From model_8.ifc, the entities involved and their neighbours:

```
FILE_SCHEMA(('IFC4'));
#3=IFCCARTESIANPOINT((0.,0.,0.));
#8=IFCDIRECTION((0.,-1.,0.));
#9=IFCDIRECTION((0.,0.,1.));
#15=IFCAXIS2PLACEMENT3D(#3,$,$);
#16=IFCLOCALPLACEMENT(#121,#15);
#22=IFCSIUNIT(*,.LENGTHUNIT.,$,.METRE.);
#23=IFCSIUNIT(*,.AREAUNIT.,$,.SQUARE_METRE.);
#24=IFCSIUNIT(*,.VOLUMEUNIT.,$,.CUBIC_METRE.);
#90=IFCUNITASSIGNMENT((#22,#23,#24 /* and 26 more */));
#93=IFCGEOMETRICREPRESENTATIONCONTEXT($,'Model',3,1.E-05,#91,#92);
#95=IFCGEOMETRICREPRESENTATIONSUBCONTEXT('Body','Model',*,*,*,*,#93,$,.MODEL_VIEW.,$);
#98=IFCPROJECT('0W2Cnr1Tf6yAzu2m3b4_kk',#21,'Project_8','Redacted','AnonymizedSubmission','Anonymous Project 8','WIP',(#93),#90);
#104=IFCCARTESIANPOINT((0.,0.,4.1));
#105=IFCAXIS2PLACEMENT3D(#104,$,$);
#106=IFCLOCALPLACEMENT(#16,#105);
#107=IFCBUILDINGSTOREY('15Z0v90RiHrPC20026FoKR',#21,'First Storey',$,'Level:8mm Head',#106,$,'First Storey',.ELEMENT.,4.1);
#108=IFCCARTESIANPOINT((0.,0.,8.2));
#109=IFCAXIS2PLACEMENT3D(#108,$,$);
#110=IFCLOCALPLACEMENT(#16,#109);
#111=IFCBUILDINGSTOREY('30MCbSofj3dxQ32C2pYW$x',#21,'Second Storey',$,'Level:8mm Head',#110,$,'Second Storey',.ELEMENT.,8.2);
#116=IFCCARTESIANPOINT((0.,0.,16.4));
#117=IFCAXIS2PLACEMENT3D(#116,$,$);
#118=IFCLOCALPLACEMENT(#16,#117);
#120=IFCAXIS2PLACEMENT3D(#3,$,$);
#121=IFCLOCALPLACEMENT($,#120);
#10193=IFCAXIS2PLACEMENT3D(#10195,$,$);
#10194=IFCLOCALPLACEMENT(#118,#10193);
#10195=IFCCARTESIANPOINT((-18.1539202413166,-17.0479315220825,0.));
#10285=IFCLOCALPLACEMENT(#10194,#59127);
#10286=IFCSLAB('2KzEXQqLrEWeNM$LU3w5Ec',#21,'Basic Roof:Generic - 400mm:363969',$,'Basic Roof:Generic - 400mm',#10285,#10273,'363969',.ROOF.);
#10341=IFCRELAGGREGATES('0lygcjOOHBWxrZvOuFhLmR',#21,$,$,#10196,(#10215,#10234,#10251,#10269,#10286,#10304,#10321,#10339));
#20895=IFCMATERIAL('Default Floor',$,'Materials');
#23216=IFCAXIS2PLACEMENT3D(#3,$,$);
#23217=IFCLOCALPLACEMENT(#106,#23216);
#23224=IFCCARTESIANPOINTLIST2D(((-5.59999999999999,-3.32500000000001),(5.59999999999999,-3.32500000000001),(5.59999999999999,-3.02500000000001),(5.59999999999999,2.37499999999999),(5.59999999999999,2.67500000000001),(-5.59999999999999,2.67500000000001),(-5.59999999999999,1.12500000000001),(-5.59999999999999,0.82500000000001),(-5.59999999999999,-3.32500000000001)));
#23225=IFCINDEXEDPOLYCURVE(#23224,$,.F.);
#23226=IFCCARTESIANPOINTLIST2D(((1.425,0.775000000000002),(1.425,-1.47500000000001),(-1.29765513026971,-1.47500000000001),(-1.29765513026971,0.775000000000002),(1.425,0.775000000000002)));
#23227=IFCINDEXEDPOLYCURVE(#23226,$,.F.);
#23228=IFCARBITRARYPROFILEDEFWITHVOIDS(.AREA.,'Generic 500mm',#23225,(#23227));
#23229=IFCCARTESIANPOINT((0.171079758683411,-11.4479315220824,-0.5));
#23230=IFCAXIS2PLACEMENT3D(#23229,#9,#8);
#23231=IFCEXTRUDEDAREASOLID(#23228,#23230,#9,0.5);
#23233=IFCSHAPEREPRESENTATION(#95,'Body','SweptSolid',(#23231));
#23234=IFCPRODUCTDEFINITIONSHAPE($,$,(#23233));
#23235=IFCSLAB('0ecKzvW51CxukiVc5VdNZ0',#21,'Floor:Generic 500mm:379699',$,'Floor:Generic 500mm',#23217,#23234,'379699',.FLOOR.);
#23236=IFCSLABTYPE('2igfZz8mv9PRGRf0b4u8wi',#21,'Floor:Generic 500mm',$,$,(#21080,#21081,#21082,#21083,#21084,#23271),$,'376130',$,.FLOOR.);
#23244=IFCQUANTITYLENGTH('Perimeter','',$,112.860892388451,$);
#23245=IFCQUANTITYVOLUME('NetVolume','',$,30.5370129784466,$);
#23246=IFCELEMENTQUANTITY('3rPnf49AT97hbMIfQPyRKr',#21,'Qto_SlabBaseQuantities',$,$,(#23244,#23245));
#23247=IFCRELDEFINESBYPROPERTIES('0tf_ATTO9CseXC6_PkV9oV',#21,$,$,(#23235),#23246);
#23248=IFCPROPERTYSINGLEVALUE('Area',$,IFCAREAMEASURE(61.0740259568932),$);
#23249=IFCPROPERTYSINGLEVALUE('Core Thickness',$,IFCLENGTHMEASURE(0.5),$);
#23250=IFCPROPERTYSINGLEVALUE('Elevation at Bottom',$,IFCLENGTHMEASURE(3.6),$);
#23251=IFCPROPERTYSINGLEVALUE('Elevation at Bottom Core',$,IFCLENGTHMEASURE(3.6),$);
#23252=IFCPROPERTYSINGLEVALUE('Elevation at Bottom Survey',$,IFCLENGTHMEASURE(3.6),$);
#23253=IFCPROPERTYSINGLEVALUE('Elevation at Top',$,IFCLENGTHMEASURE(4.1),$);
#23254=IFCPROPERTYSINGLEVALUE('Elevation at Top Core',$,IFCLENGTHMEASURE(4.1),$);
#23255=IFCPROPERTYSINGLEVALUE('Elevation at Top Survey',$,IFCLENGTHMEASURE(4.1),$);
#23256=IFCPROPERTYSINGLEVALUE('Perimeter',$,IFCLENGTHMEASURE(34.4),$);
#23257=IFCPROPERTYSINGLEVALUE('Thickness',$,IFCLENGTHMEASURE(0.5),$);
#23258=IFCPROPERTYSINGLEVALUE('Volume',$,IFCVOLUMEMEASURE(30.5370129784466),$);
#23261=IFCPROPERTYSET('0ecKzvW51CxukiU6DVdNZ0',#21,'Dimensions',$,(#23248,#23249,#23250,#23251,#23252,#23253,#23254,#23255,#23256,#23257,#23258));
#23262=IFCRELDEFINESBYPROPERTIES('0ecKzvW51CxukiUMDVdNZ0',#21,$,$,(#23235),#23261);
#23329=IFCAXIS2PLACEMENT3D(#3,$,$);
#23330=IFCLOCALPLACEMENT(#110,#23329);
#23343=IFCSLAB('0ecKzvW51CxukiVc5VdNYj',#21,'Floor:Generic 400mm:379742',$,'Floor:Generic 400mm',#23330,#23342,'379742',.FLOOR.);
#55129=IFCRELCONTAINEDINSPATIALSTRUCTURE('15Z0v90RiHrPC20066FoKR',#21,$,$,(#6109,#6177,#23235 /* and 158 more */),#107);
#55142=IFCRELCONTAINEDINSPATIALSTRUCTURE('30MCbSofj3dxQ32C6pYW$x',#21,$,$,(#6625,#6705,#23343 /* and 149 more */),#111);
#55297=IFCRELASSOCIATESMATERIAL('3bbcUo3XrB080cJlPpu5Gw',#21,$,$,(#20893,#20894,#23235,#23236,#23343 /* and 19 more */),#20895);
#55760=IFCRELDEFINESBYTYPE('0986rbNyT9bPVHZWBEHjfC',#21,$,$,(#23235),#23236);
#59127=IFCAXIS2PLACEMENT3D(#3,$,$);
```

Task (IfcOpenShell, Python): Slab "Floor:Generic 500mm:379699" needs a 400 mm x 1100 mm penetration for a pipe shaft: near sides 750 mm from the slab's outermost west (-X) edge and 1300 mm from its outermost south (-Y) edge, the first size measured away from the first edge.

```python
import numpy as np
import ifcopenshell
import ifcopenshell.api.feature
import ifcopenshell.api.geometry
import ifcopenshell.api.pset
import ifcopenshell.api.root
import ifcopenshell.geom
import ifcopenshell.util.element
import ifcopenshell.util.placement
import ifcopenshell.util.representation
import ifcopenshell.util.shape
import ifcopenshell.util.unit

model = ifcopenshell.open("model_8.ifc")
unit_scale = ifcopenshell.util.unit.calculate_unit_scale(model)
area_scale = ifcopenshell.util.unit.calculate_unit_scale(model, "AREAUNIT")
volume_scale = ifcopenshell.util.unit.calculate_unit_scale(model, "VOLUMEUNIT")
settings = ifcopenshell.geom.settings()


def volume(element):
    """Net volume in cubic metres, openings subtracted."""
    shape = ifcopenshell.geom.create_shape(settings, element)
    return ifcopenshell.util.shape.get_volume(shape.geometry)


slab = model.by_guid("0ecKzvW51CxukiVc5VdNZ0")
before = volume(slab)

# Extent in the slab's own axes, in metres. The edges named are its -X and -Y sides.
slab_shape = ifcopenshell.geom.create_shape(settings, slab)
vertices = ifcopenshell.util.shape.get_vertices(slab_shape.geometry)
x_min, y_min, bottom = vertices.min(axis=0)
top = vertices[:, 2].max()

opening = ifcopenshell.api.root.create_entity(model, ifc_class="IfcOpeningElement", name="Pipe shaft opening", predefined_type="OPENING")
context = ifcopenshell.util.representation.get_context(model, "Model", "Body", "MODEL_VIEW")
width, depth = 0.4, 1.1
outline = [(0.0, 0.0), (width, 0.0), (width, depth), (0.0, depth), (0.0, 0.0)]
# Overshoot both faces by 50 mm so the cut is clean.
shape = ifcopenshell.api.geometry.add_slab_representation(
    model, context=context, depth=top - bottom + 0.1, polyline=outline
)
ifcopenshell.api.geometry.assign_representation(model, product=opening, representation=shape)

matrix = ifcopenshell.util.placement.get_local_placement(slab.ObjectPlacement)
matrix[:, 3] = matrix @ np.append(np.array([x_min + 0.75, y_min + 1.3, bottom - 0.05]) / unit_scale, 1.0)
ifcopenshell.api.geometry.edit_object_placement(model, product=opening, matrix=matrix, is_si=False)
ifcopenshell.api.feature.add_feature(model, feature=opening, element=slab)

after = volume(slab)

# Update the slab's stored quantities.
qto = model.by_id(ifcopenshell.util.element.get_pset(slab, "Qto_SlabBaseQuantities", should_inherit=False)["id"])
ifcopenshell.api.pset.edit_qto(model, qto=qto, properties={"NetVolume": after / volume_scale})
pset = model.by_id(ifcopenshell.util.element.get_pset(slab, "Dimensions", should_inherit=False)["id"])
ifcopenshell.api.pset.edit_pset(model, pset=pset, properties={
    "Area": model.create_entity("IfcAreaMeasure", after / (top - bottom) / area_scale),
    "Volume": model.create_entity("IfcVolumeMeasure", after / volume_scale),
})

print(f"slab volume {before:.3f} -> {after:.3f} m3")

model.write("model_8_updated.ifc")
```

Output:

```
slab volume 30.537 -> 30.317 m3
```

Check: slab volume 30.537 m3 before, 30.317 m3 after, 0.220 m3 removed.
